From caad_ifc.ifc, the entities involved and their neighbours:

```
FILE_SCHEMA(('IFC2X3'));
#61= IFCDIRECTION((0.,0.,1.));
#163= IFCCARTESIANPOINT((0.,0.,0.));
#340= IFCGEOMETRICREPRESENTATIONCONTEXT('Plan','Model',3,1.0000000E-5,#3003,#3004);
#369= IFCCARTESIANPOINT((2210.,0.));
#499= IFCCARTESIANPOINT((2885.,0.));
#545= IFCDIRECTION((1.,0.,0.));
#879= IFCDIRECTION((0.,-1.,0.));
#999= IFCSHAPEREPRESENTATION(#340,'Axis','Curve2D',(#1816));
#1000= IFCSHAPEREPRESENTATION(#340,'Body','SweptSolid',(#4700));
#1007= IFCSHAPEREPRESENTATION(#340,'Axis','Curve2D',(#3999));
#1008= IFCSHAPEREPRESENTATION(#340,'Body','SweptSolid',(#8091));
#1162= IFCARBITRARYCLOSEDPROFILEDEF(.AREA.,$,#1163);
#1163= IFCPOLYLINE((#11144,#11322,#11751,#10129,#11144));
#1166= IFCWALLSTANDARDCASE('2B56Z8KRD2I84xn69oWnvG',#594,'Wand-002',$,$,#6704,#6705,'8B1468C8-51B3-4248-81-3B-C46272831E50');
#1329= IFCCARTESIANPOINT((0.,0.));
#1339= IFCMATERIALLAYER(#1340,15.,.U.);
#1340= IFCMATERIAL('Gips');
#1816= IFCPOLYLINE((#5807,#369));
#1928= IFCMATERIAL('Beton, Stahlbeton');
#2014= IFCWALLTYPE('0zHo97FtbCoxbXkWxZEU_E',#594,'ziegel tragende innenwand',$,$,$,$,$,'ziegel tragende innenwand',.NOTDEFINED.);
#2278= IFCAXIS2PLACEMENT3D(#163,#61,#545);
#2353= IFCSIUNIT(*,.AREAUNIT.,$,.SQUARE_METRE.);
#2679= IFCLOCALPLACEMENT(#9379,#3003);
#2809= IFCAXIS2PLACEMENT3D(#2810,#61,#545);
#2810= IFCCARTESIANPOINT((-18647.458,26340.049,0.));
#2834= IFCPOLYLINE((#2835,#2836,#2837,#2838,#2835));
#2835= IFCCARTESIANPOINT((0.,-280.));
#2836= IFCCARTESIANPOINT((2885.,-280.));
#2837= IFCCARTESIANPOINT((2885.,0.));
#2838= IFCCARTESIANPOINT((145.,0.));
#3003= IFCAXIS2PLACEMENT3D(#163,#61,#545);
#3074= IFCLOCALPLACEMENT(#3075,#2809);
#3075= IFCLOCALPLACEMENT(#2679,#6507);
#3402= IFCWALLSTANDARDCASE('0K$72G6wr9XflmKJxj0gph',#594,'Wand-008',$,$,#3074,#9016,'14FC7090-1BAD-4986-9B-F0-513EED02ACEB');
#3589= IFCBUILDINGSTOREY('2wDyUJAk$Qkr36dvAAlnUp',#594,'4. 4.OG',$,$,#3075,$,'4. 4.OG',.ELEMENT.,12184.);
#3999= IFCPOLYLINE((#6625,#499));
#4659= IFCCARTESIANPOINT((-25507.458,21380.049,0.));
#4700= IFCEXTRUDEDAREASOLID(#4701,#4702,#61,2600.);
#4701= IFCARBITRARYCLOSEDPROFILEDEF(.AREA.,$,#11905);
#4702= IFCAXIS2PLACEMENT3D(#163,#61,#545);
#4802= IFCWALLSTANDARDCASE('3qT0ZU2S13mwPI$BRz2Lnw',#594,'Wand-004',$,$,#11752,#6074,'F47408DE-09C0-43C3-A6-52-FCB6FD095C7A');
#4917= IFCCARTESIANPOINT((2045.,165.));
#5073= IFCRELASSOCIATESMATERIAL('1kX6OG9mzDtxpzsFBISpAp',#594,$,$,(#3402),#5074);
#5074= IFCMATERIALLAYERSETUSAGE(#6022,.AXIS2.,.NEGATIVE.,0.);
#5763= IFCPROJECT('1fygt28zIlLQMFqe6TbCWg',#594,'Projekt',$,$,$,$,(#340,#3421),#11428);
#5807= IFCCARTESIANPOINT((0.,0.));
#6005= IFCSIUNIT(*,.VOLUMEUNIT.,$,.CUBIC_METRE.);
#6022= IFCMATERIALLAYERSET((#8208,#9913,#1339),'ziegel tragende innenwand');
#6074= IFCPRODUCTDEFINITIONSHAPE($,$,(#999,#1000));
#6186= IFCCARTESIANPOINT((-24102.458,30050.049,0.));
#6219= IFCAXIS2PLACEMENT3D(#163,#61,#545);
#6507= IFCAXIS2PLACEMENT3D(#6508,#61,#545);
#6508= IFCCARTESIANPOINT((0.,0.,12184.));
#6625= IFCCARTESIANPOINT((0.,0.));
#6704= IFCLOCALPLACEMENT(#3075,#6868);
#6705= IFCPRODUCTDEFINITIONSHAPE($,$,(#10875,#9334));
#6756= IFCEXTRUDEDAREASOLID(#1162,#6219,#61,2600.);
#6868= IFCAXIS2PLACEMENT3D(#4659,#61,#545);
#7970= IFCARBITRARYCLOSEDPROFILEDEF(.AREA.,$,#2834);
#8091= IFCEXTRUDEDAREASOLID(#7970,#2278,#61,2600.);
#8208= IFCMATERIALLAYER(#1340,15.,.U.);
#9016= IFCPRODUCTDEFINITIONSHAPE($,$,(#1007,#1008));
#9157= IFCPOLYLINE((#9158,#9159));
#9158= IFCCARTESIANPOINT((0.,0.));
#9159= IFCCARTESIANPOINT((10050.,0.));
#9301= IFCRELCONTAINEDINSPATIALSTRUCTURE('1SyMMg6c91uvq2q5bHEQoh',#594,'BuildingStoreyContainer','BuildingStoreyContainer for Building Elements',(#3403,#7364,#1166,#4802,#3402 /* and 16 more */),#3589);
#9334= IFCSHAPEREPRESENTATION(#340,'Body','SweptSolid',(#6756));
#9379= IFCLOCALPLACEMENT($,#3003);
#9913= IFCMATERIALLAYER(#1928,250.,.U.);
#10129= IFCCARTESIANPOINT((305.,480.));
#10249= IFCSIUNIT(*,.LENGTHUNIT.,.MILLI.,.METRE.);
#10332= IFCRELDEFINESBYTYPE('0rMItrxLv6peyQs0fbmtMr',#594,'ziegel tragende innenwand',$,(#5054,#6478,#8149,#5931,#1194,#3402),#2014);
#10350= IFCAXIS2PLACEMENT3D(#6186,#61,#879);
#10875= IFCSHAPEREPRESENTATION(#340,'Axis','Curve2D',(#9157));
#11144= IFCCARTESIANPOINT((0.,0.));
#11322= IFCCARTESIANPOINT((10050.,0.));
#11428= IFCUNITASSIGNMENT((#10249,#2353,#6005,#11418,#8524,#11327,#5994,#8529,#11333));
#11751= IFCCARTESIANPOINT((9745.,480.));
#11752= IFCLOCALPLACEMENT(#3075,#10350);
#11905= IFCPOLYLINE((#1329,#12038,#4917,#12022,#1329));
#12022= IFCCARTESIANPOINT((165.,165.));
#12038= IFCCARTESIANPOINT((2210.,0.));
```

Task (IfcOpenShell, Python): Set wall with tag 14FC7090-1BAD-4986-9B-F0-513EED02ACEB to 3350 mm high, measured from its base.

```python
import ifcopenshell
import ifcopenshell.geom
import ifcopenshell.util.shape
import ifcopenshell.util.unit

model = ifcopenshell.open("caad_ifc.ifc")
unit_scale = ifcopenshell.util.unit.calculate_unit_scale(model)
settings = ifcopenshell.geom.settings()


def volume(element):
    """Net volume in cubic metres, openings subtracted."""
    shape = ifcopenshell.geom.create_shape(settings, element)
    return ifcopenshell.util.shape.get_volume(shape.geometry)


wall = model.by_guid("0K$72G6wr9XflmKJxj0gph")
before = volume(wall)

body = next(r for r in wall.Representation.Representations if r.RepresentationIdentifier == "Body")
solid = body.Items[0]
old_height = solid.Depth
solid.Depth = 3.35 / unit_scale
after = volume(wall)

print(f"height {old_height:g} -> {solid.Depth:g}, volume {before:.3f} -> {after:.3f} m3")

model.write("caad_ifc_v2.ifc")
```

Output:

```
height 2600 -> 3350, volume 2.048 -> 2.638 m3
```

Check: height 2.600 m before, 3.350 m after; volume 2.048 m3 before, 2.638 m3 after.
